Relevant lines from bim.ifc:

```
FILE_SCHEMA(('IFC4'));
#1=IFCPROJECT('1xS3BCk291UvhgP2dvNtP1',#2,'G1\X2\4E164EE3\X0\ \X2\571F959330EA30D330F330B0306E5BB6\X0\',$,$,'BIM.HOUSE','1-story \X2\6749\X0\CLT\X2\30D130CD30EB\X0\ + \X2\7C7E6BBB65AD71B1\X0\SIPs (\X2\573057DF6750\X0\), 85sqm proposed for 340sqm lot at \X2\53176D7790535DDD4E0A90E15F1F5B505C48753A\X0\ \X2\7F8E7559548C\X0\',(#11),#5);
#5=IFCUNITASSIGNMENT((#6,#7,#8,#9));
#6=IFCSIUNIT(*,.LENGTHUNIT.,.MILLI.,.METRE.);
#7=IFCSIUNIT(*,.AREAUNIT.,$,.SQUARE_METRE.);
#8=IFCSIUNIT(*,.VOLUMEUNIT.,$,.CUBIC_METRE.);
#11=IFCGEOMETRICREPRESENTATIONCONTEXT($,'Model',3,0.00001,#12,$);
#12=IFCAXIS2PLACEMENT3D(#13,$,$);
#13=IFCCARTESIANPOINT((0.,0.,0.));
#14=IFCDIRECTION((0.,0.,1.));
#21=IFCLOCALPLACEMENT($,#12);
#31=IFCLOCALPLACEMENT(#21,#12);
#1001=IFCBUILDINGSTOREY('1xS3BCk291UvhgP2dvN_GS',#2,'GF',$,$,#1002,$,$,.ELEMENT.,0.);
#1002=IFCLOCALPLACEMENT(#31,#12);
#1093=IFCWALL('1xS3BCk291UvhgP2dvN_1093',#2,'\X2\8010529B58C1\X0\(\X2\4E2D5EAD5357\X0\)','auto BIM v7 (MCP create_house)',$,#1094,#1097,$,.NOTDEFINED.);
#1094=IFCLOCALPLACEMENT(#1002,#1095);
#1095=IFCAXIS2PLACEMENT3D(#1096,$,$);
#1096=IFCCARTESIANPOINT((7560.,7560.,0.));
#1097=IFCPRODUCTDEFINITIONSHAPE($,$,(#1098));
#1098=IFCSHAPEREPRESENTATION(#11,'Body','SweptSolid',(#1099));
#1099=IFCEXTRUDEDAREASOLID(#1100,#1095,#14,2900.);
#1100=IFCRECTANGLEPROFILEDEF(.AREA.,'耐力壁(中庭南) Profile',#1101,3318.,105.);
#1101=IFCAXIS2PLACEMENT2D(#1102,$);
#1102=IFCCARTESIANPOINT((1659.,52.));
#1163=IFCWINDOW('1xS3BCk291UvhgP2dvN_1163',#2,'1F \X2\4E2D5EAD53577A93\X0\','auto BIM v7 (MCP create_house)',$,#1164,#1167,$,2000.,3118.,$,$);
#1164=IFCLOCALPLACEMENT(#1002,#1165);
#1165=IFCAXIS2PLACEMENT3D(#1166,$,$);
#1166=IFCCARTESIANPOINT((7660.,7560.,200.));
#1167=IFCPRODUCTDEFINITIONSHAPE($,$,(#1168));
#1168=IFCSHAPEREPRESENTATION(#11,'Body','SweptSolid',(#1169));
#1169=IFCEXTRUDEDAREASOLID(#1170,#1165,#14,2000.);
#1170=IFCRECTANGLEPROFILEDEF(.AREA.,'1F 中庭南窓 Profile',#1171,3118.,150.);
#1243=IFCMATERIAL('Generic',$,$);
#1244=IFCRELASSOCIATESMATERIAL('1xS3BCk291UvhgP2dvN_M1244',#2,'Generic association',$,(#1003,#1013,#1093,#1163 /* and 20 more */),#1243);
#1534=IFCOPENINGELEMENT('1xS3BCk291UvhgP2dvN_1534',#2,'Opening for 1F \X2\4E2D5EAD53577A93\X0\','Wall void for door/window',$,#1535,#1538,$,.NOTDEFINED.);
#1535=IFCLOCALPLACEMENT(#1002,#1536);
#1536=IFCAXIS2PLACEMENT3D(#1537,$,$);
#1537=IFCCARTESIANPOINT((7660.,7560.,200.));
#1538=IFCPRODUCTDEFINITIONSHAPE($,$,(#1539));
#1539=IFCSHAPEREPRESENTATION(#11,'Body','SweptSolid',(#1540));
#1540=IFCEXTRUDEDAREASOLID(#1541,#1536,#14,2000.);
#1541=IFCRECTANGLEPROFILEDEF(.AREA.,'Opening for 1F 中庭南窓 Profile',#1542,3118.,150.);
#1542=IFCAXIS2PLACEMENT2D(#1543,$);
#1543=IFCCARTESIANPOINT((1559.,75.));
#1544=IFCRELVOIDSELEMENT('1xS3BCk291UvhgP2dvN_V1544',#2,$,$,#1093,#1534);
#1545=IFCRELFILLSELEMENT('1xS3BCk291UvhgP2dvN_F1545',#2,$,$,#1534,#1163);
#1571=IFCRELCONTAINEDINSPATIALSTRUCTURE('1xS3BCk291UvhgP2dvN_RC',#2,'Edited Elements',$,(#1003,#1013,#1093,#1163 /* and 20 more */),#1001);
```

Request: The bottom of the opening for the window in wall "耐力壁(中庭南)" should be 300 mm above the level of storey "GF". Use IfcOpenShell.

```python
import numpy as np
import ifcopenshell
import ifcopenshell.api.geometry
import ifcopenshell.geom
import ifcopenshell.util.element
import ifcopenshell.util.placement
import ifcopenshell.util.shape
import ifcopenshell.util.unit

model = ifcopenshell.open("bim.ifc")
unit_scale = ifcopenshell.util.unit.calculate_unit_scale(model)

window = model.by_guid("1xS3BCk291UvhgP2dvN_1163")
opening = window.FillsVoids[0].RelatingOpeningElement
storey = ifcopenshell.util.element.get_container(window, ifc_class="IfcBuildingStorey")
level = ifcopenshell.util.placement.get_local_placement(storey.ObjectPlacement)[2, 3]

# The opening's origin need not be at the sill, so measure its lowest point.
shape = ifcopenshell.geom.create_shape(ifcopenshell.geom.settings(), opening)
bottom = ifcopenshell.util.shape.get_shape_bottom_elevation(shape, shape.geometry) / unit_scale
dz = level + 0.3 / unit_scale - bottom

shift = np.array([0.0, 0.0, dz])
# The window is not placed relative to its opening, so move both.
for product in (opening, window):
    matrix = ifcopenshell.util.placement.get_local_placement(product.ObjectPlacement)
    matrix[:3, 3] += shift
    ifcopenshell.api.geometry.edit_object_placement(model, product=product, matrix=matrix, is_si=False)

print(f"moved by {dz * unit_scale:+.3f} m")

model.write("bim-out.ifc")
```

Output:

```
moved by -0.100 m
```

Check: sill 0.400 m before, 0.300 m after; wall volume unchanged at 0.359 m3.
